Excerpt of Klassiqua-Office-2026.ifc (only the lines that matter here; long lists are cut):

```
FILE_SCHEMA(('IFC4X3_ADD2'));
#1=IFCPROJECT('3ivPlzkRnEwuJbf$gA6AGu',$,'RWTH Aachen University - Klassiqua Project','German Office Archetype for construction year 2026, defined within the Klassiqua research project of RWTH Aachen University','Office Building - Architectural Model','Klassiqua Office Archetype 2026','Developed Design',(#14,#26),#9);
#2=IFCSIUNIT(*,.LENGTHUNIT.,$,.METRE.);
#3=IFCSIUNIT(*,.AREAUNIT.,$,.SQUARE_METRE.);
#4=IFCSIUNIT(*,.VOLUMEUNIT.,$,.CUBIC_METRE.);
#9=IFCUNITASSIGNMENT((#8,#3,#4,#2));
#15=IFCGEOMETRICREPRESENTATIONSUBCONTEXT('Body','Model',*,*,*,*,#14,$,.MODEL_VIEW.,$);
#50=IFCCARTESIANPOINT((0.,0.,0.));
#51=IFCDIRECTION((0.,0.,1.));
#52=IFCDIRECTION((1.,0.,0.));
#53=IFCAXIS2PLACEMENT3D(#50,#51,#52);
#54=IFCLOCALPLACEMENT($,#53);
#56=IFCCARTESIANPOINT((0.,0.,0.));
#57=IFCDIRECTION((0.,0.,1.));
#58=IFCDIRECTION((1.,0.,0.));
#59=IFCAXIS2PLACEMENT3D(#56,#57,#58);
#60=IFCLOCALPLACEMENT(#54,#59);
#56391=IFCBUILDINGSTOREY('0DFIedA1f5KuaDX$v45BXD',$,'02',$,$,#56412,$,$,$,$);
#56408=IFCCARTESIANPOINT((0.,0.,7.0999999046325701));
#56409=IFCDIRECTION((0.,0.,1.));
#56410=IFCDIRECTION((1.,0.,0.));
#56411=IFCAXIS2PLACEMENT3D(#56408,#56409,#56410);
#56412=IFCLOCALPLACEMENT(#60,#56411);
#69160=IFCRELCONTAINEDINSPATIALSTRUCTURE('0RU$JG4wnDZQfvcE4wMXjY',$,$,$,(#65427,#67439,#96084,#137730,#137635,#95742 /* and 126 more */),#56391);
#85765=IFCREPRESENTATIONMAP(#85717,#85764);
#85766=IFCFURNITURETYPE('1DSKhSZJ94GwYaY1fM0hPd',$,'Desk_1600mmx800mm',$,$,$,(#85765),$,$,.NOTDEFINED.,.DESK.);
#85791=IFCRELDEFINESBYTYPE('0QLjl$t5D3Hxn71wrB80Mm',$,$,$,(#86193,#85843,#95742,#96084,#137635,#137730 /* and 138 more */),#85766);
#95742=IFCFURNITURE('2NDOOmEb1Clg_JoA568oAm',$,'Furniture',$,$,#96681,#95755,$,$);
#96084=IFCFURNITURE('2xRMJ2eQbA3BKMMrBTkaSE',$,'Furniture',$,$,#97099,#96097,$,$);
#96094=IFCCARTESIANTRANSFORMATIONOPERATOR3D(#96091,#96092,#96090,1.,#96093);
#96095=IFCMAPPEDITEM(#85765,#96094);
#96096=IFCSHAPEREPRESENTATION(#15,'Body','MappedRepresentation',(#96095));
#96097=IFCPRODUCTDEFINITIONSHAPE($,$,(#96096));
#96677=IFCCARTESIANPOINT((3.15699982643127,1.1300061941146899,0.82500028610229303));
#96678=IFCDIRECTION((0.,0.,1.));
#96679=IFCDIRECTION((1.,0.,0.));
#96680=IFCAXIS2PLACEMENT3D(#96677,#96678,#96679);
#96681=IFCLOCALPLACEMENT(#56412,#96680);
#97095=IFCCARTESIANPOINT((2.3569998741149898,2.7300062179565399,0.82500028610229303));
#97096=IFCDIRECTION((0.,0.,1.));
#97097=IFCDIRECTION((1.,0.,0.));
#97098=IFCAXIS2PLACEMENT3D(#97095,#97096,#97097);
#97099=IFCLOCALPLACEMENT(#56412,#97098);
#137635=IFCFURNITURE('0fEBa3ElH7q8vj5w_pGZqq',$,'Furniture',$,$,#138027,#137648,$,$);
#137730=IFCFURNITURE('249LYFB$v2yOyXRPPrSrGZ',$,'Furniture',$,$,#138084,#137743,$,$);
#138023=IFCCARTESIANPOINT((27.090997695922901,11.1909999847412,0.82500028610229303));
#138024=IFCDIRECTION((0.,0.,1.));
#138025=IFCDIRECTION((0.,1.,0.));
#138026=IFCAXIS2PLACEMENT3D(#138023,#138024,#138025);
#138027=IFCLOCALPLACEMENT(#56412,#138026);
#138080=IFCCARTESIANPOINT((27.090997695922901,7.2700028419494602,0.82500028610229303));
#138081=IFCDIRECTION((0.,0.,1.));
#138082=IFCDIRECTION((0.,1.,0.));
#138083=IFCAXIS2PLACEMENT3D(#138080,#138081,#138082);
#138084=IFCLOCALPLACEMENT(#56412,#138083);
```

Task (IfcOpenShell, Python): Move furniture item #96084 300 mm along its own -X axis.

```python
import ifcopenshell
import ifcopenshell.api.geometry
import ifcopenshell.util.placement

model = ifcopenshell.open("Klassiqua-Office-2026.ifc")

item = model.by_guid("2xRMJ2eQbA3BKMMrBTkaSE")
matrix = ifcopenshell.util.placement.get_local_placement(item.ObjectPlacement)
matrix[:3, 3] -= matrix[:3, 0] * 0.3
ifcopenshell.api.geometry.edit_object_placement(model, product=item, matrix=matrix, is_si=False)

print(ifcopenshell.util.placement.get_local_placement(item.ObjectPlacement).round(3) + 0.0)

model.write("Klassiqua-Office-2026_edited.ifc")
```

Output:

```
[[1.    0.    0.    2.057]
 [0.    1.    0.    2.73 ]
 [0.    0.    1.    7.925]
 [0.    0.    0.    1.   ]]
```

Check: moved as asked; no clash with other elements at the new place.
